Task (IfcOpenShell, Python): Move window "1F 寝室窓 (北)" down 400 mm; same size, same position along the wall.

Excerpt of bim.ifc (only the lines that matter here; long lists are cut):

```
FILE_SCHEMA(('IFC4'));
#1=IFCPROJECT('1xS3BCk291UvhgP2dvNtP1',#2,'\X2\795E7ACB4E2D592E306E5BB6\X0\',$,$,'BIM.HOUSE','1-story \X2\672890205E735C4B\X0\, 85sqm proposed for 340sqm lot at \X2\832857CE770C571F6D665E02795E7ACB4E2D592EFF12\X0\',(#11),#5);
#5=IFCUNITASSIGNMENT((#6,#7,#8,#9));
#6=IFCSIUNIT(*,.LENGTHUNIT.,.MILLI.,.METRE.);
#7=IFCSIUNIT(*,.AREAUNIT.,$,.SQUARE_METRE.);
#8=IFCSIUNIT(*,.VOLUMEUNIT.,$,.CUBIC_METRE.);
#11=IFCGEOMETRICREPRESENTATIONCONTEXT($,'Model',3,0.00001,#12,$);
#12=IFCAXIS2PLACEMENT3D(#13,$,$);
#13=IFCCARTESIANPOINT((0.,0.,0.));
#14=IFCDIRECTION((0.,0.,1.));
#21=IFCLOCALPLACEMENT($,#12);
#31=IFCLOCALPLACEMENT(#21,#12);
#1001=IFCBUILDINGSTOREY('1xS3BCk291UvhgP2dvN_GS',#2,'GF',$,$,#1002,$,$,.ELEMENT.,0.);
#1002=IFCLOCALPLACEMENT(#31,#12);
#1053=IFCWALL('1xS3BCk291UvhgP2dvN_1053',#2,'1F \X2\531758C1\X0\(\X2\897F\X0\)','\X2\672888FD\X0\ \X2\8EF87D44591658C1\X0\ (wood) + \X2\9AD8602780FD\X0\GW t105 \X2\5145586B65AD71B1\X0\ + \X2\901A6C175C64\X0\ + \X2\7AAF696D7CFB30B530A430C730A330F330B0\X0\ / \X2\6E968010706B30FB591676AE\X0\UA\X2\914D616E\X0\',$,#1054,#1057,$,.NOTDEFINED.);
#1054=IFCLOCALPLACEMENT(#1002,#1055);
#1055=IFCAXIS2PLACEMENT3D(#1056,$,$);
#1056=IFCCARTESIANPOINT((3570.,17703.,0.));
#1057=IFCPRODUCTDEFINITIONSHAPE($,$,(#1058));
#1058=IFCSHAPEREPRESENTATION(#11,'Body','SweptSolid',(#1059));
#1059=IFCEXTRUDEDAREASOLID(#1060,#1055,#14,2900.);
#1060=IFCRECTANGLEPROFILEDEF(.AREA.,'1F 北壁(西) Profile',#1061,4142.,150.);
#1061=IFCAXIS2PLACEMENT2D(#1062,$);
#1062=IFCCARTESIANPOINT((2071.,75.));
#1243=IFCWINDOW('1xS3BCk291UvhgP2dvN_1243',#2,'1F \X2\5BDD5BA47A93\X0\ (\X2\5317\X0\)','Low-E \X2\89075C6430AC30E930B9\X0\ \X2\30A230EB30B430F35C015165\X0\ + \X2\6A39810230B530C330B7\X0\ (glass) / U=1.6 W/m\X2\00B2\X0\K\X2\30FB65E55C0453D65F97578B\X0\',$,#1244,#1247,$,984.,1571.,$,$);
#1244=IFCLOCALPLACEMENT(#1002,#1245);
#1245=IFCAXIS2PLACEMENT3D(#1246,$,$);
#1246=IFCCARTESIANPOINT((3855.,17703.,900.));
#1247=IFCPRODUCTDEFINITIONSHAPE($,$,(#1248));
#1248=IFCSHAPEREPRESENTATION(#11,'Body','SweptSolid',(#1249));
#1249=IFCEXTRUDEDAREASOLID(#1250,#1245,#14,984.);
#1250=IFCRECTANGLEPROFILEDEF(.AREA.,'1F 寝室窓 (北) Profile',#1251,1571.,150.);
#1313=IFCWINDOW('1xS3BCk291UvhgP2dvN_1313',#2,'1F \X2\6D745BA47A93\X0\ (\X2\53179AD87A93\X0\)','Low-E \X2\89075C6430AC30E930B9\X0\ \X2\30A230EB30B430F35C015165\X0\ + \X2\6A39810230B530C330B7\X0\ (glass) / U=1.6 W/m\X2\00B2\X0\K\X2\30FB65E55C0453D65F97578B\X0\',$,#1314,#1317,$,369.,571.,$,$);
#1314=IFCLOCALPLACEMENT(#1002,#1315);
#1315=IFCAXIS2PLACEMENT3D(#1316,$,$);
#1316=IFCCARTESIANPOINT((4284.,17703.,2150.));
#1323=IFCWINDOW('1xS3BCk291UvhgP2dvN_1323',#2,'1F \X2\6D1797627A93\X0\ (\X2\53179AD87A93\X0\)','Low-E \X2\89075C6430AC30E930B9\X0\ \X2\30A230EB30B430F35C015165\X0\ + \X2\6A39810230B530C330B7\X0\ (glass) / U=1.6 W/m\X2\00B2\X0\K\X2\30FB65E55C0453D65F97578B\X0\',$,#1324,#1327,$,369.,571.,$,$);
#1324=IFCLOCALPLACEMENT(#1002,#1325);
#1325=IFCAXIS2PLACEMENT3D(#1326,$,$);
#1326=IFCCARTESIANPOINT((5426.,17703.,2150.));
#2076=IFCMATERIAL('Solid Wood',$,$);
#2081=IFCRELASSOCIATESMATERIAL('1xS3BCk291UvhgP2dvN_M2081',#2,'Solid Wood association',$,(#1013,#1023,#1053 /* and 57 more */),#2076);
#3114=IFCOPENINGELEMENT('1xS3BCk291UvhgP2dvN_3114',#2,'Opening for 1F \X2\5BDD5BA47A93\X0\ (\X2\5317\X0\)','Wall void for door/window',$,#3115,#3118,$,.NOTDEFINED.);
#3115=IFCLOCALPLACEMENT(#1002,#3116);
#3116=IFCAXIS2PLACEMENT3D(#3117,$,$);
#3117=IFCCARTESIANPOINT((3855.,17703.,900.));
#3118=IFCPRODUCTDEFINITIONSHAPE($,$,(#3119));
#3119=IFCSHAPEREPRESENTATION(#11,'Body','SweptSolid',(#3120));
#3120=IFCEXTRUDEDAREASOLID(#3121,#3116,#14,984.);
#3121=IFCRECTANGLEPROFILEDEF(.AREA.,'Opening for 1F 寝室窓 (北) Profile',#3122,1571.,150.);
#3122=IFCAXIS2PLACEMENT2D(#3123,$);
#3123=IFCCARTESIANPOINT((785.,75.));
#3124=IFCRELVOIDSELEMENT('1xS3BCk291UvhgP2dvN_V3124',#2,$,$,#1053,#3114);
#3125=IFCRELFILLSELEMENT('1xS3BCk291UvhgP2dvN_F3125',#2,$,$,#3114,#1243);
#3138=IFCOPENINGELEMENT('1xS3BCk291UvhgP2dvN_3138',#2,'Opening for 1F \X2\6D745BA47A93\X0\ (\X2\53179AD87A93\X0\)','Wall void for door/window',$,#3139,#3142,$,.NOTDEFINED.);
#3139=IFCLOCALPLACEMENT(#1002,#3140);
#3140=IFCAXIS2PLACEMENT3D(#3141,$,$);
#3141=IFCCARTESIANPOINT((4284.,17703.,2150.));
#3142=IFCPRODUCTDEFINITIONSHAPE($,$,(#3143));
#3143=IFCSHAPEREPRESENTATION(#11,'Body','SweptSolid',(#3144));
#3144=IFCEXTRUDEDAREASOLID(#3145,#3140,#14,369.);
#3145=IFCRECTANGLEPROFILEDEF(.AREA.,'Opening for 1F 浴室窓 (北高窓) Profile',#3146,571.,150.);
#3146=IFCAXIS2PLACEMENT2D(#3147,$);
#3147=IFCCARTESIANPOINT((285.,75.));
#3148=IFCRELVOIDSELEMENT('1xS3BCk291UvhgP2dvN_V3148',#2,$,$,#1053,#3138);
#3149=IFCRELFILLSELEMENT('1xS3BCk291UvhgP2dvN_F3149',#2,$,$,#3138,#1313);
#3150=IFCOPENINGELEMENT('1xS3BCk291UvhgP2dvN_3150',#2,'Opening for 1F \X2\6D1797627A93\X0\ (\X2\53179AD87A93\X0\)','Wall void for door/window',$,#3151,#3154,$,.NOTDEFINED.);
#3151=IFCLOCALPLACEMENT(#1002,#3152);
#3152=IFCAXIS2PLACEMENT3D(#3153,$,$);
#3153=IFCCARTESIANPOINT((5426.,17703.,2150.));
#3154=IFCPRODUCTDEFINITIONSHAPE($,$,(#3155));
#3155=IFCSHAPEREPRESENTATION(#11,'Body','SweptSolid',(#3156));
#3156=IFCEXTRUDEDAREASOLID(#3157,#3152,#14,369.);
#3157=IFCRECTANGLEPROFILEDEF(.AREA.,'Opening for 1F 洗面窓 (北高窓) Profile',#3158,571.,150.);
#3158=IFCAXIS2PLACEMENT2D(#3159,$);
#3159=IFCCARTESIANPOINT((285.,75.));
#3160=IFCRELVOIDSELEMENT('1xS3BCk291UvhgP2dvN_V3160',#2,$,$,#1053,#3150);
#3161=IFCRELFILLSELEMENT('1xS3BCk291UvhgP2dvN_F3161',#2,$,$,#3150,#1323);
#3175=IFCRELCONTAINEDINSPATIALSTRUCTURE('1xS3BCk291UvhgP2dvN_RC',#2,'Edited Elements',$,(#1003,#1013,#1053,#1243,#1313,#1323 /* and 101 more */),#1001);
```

```python
import numpy as np
import ifcopenshell
import ifcopenshell.api.geometry
import ifcopenshell.util.placement
import ifcopenshell.util.unit

model = ifcopenshell.open("bim.ifc")
unit_scale = ifcopenshell.util.unit.calculate_unit_scale(model)

window = model.by_id(1243)
opening = window.FillsVoids[0].RelatingOpeningElement
dz = -0.4 / unit_scale

shift = np.array([0.0, 0.0, dz])
# The window is not placed relative to its opening, so move both.
for product in (opening, window):
    matrix = ifcopenshell.util.placement.get_local_placement(product.ObjectPlacement)
    matrix[:3, 3] += shift
    ifcopenshell.api.geometry.edit_object_placement(model, product=product, matrix=matrix, is_si=False)

print(f"moved by {dz * unit_scale:+.3f} m")

model.write("bim_v2.ifc")
```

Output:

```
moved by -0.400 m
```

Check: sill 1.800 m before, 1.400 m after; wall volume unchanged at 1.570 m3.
